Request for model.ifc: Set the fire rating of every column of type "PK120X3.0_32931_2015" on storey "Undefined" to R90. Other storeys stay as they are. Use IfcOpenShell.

First a look at what the model holds.

```python
import ifcopenshell
import ifcopenshell.util.element

model = ifcopenshell.open("model.ifc")
print(model.schema)
storey = next(s for s in model.by_type("IfcBuildingStorey") if s.Name == "Undefined")
columns = [e for e in ifcopenshell.util.element.get_decomposition(storey) if e.is_a("IfcColumn")]
seen = {}
for e in columns:
    element_type = ifcopenshell.util.element.get_type(e)
    key = (element_type.Name if element_type != e and element_type else None, ifcopenshell.util.element.get_pset(e, "Pset_ColumnCommon", "FireRating"))
    seen[key] = seen.get(key, 0) + 1
for (name, value), count in sorted(seen.items(), key=str):
    print(count, "x", name, "|", value)
```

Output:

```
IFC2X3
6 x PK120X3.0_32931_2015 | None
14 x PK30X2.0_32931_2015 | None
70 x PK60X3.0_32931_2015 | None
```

```python
import ifcopenshell
import ifcopenshell.api.pset
import ifcopenshell.util.element

model = ifcopenshell.open("model.ifc")

storey = next(s for s in model.by_type("IfcBuildingStorey") if s.Name == "Undefined")
columns = [e for e in ifcopenshell.util.element.get_decomposition(storey) if e.is_a("IfcColumn")]

count = 0
for e in columns:
    element_type = ifcopenshell.util.element.get_type(e)
    if element_type in (None, e) or element_type.Name != "PK120X3.0_32931_2015":
        continue
    found = ifcopenshell.util.element.get_pset(e, "Pset_ColumnCommon", should_inherit=False)
    if found:
        pset = model.by_id(found["id"])
        if len(ifcopenshell.util.element.get_elements_by_pset(pset)) > 1:
            pset = ifcopenshell.api.pset.unshare_pset(model, products=[e], pset=pset)[0]
    else:
        pset = ifcopenshell.api.pset.add_pset(model, product=e, name="Pset_ColumnCommon")
    ifcopenshell.api.pset.edit_pset(model, pset=pset, properties={"FireRating": "R90"})
    count += 1

print(count, "columns updated")

model.write("model_edited.ifc")
```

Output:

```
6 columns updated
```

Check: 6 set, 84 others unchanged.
